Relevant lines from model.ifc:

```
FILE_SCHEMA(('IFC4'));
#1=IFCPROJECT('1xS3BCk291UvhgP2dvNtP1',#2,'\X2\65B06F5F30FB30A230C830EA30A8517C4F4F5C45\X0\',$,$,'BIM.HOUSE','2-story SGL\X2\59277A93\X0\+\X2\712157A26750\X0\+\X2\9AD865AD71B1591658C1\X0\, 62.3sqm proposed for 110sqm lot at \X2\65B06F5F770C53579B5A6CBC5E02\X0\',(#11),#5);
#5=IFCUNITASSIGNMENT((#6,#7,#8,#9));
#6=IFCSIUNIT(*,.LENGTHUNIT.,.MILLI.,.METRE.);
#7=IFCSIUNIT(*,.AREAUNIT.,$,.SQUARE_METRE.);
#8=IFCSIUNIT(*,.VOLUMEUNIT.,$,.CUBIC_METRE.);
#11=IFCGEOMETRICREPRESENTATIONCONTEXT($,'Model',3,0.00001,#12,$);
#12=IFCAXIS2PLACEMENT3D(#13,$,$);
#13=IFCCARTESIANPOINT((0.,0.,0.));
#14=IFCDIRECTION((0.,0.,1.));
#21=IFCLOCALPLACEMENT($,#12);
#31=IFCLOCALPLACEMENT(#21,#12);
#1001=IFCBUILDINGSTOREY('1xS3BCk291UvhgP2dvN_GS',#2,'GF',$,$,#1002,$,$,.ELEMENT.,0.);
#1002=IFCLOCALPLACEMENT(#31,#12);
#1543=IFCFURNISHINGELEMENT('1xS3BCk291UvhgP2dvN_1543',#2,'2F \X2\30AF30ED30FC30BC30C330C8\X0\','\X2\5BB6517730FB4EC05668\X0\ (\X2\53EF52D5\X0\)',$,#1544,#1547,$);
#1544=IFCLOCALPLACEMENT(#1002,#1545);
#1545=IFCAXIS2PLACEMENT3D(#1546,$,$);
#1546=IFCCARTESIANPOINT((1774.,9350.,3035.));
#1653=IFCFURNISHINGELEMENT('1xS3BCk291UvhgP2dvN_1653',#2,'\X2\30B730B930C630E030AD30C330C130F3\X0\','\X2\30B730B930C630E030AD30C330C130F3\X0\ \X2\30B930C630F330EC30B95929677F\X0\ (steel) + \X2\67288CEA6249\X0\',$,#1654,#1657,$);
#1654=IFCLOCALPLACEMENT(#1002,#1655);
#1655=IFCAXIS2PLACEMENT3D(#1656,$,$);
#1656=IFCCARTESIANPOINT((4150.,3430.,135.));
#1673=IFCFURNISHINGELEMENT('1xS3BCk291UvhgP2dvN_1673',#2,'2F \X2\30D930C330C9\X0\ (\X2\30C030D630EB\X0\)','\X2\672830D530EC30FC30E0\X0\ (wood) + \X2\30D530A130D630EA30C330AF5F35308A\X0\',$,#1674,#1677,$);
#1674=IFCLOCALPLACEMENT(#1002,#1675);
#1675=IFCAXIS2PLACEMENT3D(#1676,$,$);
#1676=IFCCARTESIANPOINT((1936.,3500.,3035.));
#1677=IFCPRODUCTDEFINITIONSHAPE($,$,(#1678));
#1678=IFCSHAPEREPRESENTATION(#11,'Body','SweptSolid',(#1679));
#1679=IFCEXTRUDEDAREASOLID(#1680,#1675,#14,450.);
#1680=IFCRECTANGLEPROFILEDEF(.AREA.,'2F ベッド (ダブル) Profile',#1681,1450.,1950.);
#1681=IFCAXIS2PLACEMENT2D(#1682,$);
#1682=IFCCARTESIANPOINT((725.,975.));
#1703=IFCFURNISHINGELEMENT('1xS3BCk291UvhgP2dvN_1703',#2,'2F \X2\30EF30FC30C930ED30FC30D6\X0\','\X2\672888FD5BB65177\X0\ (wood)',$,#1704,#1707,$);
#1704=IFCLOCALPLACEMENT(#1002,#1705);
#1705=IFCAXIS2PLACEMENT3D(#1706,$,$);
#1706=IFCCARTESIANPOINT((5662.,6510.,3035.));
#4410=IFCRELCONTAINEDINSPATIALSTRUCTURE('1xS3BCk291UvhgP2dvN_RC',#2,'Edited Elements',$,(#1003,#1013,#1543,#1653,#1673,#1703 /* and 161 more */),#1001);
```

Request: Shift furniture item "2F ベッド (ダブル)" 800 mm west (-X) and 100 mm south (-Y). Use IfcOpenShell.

```python
import ifcopenshell
import ifcopenshell.api.geometry
import ifcopenshell.util.placement
import ifcopenshell.util.unit

model = ifcopenshell.open("model.ifc")
unit_scale = ifcopenshell.util.unit.calculate_unit_scale(model)

item = model.by_guid("1xS3BCk291UvhgP2dvN_1673")
matrix = ifcopenshell.util.placement.get_local_placement(item.ObjectPlacement)
matrix[0, 3] -= 0.8 / unit_scale
matrix[1, 3] -= 0.1 / unit_scale
ifcopenshell.api.geometry.edit_object_placement(model, product=item, matrix=matrix, is_si=False)

print(ifcopenshell.util.placement.get_local_placement(item.ObjectPlacement).round(3) + 0.0)

model.write("model_v2.ifc")
```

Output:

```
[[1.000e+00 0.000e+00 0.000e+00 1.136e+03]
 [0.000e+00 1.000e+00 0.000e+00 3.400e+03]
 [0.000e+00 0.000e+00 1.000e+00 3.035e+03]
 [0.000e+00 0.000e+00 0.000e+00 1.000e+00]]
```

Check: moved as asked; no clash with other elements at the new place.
